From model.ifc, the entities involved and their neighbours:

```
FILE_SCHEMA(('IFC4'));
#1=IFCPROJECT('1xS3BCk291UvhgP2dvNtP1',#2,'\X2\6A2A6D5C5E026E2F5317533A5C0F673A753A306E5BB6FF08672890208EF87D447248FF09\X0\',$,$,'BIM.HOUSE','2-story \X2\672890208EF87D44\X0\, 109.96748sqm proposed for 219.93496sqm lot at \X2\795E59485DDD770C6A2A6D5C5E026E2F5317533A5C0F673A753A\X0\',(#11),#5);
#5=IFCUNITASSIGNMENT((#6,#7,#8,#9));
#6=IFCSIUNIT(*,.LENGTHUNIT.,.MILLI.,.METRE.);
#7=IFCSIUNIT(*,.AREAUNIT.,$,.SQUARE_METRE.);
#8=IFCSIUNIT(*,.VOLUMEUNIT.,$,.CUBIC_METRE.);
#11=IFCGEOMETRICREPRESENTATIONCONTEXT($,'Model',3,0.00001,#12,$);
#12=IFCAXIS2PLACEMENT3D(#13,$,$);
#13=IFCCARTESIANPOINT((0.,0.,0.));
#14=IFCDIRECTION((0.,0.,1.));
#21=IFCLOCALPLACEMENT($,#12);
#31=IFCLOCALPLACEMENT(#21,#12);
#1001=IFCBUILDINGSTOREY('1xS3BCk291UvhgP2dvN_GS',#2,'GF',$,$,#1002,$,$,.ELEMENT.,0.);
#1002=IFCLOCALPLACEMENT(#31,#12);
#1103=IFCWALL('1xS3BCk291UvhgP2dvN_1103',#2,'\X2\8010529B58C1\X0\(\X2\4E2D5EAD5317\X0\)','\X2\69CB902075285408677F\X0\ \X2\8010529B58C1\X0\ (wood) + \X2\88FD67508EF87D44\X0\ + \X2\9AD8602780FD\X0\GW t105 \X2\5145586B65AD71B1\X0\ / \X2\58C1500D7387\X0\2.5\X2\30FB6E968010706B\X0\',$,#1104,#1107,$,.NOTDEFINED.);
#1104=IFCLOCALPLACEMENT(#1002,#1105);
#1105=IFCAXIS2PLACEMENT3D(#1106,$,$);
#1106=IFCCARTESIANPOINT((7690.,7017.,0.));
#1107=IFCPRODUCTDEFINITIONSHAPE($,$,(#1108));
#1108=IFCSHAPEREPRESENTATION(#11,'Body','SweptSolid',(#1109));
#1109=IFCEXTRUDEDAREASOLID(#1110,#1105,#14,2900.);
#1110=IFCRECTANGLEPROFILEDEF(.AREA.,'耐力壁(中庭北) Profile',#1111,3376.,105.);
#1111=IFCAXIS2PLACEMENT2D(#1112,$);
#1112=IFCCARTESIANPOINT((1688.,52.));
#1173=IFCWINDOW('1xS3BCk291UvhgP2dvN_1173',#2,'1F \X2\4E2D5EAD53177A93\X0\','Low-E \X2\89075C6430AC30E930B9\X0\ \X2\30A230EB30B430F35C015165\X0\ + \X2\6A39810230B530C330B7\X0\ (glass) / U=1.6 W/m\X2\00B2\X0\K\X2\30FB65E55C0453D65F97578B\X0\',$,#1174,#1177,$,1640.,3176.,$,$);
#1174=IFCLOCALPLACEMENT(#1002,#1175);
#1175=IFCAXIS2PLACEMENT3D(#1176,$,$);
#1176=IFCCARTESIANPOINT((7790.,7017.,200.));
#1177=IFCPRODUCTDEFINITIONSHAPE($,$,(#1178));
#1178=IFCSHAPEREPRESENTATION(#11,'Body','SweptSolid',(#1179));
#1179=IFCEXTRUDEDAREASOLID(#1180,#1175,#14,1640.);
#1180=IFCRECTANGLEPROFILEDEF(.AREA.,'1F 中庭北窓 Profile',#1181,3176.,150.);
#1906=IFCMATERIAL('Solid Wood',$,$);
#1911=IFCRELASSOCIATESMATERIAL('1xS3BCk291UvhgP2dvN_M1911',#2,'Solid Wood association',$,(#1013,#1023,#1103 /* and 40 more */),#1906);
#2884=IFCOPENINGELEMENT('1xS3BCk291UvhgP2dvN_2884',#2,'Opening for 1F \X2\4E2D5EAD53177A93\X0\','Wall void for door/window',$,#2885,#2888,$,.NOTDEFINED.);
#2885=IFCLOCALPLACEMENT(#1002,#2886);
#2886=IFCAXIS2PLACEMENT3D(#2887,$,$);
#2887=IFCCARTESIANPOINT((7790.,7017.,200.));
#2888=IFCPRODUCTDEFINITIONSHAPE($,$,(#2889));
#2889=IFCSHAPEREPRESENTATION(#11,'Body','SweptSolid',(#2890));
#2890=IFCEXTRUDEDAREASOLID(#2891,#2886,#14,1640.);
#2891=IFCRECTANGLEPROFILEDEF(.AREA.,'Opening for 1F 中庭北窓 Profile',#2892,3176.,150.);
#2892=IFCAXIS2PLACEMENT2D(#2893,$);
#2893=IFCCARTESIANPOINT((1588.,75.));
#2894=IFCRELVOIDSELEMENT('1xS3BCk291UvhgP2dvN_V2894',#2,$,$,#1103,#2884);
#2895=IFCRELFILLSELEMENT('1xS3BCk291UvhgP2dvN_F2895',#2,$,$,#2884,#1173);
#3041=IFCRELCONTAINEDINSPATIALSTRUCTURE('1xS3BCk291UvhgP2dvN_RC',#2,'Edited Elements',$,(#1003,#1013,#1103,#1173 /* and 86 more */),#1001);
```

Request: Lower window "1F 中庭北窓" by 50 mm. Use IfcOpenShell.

```python
import numpy as np
import ifcopenshell
import ifcopenshell.api.geometry
import ifcopenshell.util.placement
import ifcopenshell.util.unit

model = ifcopenshell.open("model.ifc")
unit_scale = ifcopenshell.util.unit.calculate_unit_scale(model)

window = model.by_guid("1xS3BCk291UvhgP2dvN_1173")
opening = window.FillsVoids[0].RelatingOpeningElement
dz = -0.05 / unit_scale

shift = np.array([0.0, 0.0, dz])
# The window is not placed relative to its opening, so move both.
for product in (opening, window):
    matrix = ifcopenshell.util.placement.get_local_placement(product.ObjectPlacement)
    matrix[:3, 3] += shift
    ifcopenshell.api.geometry.edit_object_placement(model, product=product, matrix=matrix, is_si=False)

print(f"moved by {dz * unit_scale:+.3f} m")

model.write("model_rev.ifc")
```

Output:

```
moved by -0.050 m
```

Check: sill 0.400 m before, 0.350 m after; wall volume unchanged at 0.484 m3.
